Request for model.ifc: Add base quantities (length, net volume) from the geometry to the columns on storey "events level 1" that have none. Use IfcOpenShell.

First a look at what the model holds.

```python
import ifcopenshell
import ifcopenshell.util.element
import ifcopenshell.util.unit

model = ifcopenshell.open("model.ifc")
print(model.schema)
for unit_type in ("LENGTHUNIT", "AREAUNIT", "VOLUMEUNIT"):
    print(unit_type, ifcopenshell.util.unit.calculate_unit_scale(model, unit_type))
storey = next(s for s in model.by_type("IfcBuildingStorey") if s.Name == "events level 1")
columns = [e for e in ifcopenshell.util.element.get_decomposition(storey) if e.is_a("IfcColumn")]
for e in sorted(columns, key=lambda e: e.id()):
    print(e.id(), e.is_a(), e.Name, list(ifcopenshell.util.element.get_psets(e, qtos_only=True)), sep=" | ")
```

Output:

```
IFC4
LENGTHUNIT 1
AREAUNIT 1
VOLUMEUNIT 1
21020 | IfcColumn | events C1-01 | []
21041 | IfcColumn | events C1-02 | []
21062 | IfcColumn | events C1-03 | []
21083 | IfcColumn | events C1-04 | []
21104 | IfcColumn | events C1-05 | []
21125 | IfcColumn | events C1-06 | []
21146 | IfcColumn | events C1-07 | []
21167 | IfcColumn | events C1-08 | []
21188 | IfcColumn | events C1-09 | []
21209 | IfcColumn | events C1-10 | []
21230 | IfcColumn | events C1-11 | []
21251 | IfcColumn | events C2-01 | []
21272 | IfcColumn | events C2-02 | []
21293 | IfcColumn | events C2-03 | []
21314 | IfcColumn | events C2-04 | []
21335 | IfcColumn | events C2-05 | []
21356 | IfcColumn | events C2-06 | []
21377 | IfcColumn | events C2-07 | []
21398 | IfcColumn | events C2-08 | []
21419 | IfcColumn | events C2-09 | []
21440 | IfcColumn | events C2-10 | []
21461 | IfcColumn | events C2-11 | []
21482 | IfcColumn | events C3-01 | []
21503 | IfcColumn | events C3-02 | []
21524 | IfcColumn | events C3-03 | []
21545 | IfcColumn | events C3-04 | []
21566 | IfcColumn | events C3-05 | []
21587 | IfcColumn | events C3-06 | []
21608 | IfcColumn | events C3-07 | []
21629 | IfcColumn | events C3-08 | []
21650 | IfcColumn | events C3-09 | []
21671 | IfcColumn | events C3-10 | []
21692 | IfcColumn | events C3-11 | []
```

```python
import ifcopenshell
import ifcopenshell.api.pset
import ifcopenshell.geom
import ifcopenshell.util.element
import ifcopenshell.util.shape
import ifcopenshell.util.unit

model = ifcopenshell.open("model.ifc")
unit_scale = ifcopenshell.util.unit.calculate_unit_scale(model)
volume_scale = ifcopenshell.util.unit.calculate_unit_scale(model, "VOLUMEUNIT")
settings = ifcopenshell.geom.settings()

storey = next(s for s in model.by_type("IfcBuildingStorey") if s.Name == "events level 1")
columns = [e for e in ifcopenshell.util.element.get_decomposition(storey) if e.is_a("IfcColumn")]

for e in sorted(columns, key=lambda e: e.id()):
    if ifcopenshell.util.element.get_psets(e, qtos_only=True, should_inherit=False):
        continue
    # Geometry comes back in metres, in the element's own axes.
    shape = ifcopenshell.geom.create_shape(settings, e)
    values = {
        "Length": ifcopenshell.util.shape.get_z(shape.geometry) / unit_scale,
        "NetVolume": ifcopenshell.util.shape.get_volume(shape.geometry) / volume_scale,
    }
    qto = ifcopenshell.api.pset.add_qto(model, product=e, name="Qto_ColumnBaseQuantities")
    ifcopenshell.api.pset.edit_qto(model, qto=qto, properties=values)
    print(e.id(), {k: round(v, 3) for k, v in values.items()})

model.write("model_v2.ifc")
```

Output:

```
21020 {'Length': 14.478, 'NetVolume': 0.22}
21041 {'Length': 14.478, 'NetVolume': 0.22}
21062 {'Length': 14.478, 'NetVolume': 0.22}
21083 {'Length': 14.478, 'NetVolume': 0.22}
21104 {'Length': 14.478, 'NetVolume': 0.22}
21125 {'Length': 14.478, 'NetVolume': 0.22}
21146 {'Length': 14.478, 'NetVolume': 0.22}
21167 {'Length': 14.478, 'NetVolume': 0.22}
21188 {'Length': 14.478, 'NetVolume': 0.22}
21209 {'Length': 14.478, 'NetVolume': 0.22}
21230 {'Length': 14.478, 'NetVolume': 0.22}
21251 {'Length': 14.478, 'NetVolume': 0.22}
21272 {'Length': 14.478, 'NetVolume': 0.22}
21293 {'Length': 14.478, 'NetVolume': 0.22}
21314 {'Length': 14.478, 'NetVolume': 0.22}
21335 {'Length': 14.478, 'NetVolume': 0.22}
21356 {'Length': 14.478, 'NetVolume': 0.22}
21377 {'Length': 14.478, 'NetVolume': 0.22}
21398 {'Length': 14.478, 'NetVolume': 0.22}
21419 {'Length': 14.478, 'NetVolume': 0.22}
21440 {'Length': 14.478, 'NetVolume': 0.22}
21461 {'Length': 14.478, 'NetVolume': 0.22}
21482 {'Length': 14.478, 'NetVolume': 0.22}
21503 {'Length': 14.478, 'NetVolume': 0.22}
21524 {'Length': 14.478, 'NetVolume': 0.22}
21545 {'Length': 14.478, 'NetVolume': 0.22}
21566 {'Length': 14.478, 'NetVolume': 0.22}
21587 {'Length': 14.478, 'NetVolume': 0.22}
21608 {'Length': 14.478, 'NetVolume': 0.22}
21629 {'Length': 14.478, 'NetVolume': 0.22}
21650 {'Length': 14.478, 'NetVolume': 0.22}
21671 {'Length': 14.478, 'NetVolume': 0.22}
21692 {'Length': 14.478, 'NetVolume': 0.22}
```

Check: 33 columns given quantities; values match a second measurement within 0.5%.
